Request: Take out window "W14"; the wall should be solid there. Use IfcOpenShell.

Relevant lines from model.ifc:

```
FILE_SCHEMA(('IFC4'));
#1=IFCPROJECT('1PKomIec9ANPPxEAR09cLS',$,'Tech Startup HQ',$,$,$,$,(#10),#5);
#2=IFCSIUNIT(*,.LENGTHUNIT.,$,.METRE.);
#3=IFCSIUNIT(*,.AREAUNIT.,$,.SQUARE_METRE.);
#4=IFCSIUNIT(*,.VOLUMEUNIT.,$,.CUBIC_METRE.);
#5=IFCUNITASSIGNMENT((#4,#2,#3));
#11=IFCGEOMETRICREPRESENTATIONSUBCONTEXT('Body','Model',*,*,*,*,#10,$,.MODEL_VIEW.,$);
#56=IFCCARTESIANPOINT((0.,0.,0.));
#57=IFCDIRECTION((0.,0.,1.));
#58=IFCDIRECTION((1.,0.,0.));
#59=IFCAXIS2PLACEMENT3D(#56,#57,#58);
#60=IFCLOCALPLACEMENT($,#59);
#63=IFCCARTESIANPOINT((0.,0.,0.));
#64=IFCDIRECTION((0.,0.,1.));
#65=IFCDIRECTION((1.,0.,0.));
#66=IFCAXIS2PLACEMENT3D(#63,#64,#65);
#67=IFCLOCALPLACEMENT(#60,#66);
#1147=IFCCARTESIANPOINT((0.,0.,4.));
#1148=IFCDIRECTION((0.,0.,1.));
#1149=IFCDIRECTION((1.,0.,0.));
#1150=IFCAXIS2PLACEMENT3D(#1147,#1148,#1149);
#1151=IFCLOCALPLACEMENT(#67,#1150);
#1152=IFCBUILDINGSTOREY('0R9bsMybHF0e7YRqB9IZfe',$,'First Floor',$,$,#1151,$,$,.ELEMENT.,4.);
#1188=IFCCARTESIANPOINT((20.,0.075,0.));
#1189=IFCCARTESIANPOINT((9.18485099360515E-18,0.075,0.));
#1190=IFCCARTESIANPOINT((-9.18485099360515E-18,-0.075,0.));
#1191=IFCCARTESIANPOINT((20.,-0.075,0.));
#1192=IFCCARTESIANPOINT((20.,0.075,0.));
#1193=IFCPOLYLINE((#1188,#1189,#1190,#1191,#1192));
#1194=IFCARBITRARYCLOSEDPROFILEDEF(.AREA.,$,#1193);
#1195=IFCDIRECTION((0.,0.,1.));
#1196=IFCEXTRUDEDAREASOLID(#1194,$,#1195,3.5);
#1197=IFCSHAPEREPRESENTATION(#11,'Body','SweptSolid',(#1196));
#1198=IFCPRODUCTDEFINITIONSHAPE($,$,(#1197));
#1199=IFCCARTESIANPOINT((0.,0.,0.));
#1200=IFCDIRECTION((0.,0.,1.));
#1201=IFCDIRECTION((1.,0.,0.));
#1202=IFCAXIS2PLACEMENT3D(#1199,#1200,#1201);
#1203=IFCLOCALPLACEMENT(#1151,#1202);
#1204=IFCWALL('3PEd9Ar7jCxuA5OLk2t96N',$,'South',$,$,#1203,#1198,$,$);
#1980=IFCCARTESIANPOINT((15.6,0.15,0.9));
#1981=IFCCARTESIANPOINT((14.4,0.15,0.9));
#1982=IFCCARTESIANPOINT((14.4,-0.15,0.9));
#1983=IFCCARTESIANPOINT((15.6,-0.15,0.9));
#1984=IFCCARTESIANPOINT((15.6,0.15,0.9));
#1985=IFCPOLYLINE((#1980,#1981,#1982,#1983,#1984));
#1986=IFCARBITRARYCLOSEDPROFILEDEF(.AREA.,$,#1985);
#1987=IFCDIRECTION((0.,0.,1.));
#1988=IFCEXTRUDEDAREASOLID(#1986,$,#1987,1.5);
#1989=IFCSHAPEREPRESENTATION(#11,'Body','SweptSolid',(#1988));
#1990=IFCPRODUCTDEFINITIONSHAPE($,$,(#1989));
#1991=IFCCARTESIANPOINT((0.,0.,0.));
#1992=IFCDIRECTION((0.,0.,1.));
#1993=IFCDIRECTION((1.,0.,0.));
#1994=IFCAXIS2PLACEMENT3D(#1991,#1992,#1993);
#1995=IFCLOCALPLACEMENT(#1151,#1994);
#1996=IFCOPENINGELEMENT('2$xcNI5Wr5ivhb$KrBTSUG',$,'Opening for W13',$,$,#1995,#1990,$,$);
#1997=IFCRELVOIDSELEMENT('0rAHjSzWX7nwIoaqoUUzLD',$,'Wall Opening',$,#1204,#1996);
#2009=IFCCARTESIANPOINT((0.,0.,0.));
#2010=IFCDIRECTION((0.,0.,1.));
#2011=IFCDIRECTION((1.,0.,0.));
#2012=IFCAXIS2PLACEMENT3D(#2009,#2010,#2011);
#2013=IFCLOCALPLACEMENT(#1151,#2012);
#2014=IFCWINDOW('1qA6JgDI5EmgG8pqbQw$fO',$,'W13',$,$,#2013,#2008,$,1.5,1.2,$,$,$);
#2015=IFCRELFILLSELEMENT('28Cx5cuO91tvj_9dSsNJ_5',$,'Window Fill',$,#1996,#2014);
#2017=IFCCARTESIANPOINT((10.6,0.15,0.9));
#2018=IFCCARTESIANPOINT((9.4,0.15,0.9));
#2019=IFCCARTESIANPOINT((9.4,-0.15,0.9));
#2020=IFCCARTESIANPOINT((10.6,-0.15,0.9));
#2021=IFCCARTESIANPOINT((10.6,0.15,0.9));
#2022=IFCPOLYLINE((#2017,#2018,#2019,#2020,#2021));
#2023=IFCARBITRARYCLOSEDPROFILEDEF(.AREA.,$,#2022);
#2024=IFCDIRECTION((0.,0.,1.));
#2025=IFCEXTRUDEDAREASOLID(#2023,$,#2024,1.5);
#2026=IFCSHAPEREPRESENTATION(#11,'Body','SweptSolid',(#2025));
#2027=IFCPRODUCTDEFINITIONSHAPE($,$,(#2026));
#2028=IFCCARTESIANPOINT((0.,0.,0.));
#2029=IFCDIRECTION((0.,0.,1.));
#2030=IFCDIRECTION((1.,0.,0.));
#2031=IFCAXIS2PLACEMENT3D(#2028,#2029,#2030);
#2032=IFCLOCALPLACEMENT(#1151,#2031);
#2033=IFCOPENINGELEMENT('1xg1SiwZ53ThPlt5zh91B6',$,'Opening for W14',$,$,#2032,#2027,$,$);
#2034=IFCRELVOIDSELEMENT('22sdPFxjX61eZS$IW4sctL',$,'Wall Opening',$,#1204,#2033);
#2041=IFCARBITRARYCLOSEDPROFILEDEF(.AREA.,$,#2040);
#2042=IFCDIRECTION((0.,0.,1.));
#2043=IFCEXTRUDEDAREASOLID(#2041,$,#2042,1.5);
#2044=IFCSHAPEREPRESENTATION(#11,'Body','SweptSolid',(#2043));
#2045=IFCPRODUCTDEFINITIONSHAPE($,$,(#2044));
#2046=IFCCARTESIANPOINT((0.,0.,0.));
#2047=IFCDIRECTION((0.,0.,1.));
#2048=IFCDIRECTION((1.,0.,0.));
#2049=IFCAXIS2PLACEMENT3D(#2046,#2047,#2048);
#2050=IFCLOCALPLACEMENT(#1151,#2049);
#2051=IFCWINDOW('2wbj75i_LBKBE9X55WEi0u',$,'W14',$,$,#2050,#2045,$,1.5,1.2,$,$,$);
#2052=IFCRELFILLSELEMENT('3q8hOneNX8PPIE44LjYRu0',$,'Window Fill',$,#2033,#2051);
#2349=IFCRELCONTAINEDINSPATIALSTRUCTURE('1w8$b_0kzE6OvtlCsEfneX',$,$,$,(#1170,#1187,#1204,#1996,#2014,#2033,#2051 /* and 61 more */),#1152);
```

```python
import ifcopenshell
import ifcopenshell.api.feature
import ifcopenshell.api.root
import ifcopenshell.geom
import ifcopenshell.util.shape

model = ifcopenshell.open("model.ifc")
settings = ifcopenshell.geom.settings()


def volume(element):
    """Net volume in cubic metres, openings subtracted."""
    shape = ifcopenshell.geom.create_shape(settings, element)
    return ifcopenshell.util.shape.get_volume(shape.geometry)


window = model.by_guid("2wbj75i_LBKBE9X55WEi0u")
opening = window.FillsVoids[0].RelatingOpeningElement
wall = opening.VoidsElements[0].RelatingBuildingElement
before = volume(wall)

ifcopenshell.api.root.remove_product(model, product=window)
ifcopenshell.api.feature.remove_feature(model, feature=opening)

after = volume(wall)

print(f"wall volume {before:.3f} -> {after:.3f} m3")

model.write("model-out.ifc")
```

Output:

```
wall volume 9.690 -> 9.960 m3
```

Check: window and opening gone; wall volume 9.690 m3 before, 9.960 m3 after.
